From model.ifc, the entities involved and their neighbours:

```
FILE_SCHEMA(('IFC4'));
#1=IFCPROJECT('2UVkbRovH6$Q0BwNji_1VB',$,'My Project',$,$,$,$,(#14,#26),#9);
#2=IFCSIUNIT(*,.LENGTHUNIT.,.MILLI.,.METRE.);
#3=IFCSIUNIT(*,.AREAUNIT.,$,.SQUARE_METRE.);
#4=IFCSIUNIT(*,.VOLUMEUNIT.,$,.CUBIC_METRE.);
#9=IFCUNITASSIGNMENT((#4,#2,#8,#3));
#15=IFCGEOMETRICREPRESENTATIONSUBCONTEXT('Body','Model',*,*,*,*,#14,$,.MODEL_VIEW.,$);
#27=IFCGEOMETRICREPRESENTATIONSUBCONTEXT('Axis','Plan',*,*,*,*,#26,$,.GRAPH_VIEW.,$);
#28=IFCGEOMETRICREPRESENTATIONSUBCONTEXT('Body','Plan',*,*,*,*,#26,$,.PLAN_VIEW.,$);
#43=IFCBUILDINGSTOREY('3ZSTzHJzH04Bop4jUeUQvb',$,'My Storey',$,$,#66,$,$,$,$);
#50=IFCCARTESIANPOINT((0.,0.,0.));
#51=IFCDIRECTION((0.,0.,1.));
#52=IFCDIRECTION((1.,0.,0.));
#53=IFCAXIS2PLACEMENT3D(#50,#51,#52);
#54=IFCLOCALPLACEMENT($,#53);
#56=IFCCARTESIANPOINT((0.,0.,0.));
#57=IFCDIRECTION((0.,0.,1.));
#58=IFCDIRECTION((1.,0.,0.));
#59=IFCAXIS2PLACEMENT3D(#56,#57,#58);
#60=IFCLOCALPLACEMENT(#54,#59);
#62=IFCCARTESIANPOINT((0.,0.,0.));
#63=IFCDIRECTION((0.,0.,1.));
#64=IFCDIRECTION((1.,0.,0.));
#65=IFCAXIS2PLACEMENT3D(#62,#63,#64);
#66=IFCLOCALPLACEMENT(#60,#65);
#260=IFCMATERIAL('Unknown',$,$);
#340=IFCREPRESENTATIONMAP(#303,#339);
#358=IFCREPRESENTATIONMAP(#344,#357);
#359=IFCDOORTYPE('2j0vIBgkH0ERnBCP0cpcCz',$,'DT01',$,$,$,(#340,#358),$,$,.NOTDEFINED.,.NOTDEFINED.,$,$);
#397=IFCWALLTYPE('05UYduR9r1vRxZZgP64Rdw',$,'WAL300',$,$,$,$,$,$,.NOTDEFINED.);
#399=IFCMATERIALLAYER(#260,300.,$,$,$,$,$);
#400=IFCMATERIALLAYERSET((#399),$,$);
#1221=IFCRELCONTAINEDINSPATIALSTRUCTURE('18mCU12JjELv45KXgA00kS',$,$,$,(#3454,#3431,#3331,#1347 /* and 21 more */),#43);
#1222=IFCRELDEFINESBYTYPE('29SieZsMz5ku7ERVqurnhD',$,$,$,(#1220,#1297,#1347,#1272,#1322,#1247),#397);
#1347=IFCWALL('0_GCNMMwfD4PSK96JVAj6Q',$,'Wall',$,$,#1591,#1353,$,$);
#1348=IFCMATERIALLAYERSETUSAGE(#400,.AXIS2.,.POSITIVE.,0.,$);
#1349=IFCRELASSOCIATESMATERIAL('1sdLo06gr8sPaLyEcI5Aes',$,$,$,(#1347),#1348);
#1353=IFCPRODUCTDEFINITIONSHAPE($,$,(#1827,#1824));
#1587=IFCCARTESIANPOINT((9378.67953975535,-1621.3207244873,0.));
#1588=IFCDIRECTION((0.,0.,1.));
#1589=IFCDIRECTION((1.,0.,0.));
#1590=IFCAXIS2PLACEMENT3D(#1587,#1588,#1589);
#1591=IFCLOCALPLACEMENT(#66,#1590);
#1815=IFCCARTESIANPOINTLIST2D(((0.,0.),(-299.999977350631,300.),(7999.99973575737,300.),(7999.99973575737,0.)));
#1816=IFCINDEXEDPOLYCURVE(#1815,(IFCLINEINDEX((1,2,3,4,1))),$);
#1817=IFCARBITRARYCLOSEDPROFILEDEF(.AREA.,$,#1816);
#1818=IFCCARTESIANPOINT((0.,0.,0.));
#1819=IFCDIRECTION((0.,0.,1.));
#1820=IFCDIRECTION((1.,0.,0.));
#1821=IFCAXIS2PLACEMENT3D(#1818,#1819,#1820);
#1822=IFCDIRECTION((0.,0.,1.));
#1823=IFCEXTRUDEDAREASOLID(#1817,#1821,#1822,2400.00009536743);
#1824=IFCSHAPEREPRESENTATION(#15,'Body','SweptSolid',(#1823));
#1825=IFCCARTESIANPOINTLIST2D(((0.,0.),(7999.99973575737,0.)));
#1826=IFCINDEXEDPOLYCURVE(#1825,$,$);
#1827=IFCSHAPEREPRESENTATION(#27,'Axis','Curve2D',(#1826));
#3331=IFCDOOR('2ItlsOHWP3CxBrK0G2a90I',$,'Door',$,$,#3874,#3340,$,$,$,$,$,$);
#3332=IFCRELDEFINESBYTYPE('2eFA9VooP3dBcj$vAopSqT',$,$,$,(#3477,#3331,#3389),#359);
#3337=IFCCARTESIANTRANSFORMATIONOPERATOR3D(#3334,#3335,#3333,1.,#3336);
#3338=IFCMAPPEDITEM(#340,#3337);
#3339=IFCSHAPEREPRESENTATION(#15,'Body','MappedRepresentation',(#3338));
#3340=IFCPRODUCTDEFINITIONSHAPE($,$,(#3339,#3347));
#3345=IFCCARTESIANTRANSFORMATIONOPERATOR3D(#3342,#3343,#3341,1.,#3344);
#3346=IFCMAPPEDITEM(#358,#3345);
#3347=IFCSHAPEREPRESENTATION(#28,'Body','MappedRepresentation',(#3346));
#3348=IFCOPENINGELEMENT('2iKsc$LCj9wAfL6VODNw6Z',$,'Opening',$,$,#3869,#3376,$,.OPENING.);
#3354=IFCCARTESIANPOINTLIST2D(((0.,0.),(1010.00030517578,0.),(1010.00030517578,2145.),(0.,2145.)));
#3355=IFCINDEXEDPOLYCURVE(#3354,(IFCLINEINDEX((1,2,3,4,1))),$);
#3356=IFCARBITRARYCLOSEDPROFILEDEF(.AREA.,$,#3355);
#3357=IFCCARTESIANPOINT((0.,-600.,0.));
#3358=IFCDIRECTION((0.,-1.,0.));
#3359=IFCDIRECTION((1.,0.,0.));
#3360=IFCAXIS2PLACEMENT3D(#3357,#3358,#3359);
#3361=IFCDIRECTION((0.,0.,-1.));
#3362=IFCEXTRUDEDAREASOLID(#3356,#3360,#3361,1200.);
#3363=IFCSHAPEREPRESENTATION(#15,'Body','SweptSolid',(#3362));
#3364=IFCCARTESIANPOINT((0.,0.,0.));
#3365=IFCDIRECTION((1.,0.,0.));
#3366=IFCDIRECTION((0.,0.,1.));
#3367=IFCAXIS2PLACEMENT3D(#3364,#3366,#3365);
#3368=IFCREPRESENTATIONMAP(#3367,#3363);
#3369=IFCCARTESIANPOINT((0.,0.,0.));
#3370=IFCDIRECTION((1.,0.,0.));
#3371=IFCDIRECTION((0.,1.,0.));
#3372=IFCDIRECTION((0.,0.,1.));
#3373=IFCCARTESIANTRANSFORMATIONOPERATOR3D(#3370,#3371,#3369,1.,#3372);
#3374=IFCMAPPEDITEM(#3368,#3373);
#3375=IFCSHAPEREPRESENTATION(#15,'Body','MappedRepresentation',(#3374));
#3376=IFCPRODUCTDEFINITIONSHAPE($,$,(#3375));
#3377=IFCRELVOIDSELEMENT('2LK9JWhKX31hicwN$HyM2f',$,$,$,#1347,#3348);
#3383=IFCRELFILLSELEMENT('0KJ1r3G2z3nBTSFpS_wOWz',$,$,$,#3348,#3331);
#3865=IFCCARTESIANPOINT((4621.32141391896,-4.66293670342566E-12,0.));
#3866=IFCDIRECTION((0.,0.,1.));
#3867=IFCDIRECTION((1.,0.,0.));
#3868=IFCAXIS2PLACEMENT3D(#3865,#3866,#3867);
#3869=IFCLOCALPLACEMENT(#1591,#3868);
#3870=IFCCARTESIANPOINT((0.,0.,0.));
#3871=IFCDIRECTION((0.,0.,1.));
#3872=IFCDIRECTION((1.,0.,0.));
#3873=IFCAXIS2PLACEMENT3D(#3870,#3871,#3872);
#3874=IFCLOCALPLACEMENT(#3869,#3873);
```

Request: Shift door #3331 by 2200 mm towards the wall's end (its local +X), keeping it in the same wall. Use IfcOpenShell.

```python
import ifcopenshell
import ifcopenshell.api.geometry
import ifcopenshell.util.placement
import ifcopenshell.util.unit

model = ifcopenshell.open("model.ifc")
unit_scale = ifcopenshell.util.unit.calculate_unit_scale(model)

door = model.by_id(3331)
opening = door.FillsVoids[0].RelatingOpeningElement
wall = opening.VoidsElements[0].RelatingBuildingElement

wall_matrix = ifcopenshell.util.placement.get_local_placement(wall.ObjectPlacement)
shift = wall_matrix[:3, 0] * 2.2 / unit_scale
before = ifcopenshell.util.placement.get_local_placement(door.ObjectPlacement)[:3, 3].copy()

# The door is placed relative to its opening, so it follows when the opening moves.
matrix = ifcopenshell.util.placement.get_local_placement(opening.ObjectPlacement)
matrix[:3, 3] += shift
ifcopenshell.api.geometry.edit_object_placement(
    model, product=opening, matrix=matrix, is_si=False, should_transform_children=True
)

after = ifcopenshell.util.placement.get_local_placement(door.ObjectPlacement)[:3, 3]
print("door moved by", (after - before).round(3) + 0.0)

model.write("model-out.ifc")
```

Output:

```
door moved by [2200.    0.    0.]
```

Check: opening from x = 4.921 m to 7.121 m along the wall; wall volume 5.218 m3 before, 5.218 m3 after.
